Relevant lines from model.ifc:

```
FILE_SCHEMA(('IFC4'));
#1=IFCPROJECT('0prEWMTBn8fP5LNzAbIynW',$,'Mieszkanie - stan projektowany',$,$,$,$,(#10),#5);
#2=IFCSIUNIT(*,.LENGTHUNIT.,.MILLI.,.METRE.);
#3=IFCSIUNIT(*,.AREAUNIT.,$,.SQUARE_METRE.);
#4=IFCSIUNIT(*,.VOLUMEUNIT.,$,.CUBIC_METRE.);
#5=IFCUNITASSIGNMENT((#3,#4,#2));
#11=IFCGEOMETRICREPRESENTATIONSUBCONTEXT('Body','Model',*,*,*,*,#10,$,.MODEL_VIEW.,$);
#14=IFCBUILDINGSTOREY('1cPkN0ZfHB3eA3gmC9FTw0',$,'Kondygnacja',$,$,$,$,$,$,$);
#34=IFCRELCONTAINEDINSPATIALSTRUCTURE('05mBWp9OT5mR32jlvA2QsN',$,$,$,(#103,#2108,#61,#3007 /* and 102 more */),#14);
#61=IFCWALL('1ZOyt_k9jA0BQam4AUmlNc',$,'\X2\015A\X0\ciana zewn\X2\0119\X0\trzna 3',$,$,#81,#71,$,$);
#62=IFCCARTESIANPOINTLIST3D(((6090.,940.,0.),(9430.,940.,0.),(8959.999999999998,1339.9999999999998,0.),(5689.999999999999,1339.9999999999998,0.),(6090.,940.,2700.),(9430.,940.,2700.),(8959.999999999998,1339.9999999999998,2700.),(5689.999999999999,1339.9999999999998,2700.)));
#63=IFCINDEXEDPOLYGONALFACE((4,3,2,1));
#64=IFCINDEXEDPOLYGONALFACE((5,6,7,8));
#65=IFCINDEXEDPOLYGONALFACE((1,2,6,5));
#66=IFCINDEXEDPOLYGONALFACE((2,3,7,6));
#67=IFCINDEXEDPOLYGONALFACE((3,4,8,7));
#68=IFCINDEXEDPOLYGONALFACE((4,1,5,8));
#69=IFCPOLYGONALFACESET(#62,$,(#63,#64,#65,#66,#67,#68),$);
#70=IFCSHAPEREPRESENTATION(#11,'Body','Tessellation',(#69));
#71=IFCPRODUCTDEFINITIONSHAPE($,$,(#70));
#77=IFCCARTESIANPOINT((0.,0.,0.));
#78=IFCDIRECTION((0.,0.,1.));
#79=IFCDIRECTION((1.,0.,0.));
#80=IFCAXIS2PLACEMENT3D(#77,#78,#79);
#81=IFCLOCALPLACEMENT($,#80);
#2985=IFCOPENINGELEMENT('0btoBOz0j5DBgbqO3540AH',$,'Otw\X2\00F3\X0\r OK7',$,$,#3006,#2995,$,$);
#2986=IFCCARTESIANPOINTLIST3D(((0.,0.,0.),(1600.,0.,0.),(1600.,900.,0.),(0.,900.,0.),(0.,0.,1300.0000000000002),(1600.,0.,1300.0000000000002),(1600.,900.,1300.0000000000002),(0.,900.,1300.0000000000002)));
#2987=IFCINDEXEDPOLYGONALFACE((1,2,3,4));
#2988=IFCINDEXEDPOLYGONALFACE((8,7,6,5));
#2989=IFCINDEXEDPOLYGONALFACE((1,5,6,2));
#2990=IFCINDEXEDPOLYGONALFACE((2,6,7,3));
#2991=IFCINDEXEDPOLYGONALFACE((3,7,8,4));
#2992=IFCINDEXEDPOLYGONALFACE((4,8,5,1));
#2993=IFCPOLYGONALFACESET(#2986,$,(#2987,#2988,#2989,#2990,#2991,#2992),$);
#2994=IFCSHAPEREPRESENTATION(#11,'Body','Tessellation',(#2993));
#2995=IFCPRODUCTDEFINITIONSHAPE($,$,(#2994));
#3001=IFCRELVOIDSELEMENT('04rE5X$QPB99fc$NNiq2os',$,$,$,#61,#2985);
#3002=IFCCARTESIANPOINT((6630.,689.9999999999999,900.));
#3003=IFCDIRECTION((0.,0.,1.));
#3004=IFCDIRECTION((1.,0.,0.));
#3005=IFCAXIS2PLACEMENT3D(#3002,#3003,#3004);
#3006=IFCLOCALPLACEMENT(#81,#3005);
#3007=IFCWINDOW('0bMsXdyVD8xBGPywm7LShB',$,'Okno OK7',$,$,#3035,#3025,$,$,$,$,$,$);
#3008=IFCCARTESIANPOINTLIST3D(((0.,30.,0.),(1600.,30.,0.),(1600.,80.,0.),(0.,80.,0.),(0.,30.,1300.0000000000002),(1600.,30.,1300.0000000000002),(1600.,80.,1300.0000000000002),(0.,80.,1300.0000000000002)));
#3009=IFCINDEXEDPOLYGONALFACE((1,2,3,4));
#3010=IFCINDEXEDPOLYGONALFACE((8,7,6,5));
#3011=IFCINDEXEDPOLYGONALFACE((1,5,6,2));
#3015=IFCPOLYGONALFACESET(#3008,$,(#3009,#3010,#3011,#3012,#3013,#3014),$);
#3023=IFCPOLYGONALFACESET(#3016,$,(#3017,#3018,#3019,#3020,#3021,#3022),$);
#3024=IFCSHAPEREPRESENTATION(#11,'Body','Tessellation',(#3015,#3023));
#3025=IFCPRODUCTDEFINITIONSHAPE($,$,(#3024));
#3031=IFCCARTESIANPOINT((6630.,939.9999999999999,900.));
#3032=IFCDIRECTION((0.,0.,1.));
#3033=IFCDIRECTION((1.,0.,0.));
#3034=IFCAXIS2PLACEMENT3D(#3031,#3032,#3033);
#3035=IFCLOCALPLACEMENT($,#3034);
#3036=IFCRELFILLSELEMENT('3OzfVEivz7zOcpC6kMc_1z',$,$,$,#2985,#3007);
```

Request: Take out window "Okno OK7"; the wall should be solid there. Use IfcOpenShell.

```python
import ifcopenshell
import ifcopenshell.api.feature
import ifcopenshell.api.root
import ifcopenshell.geom
import ifcopenshell.util.shape

model = ifcopenshell.open("model.ifc")
settings = ifcopenshell.geom.settings()


def volume(element):
    """Net volume in cubic metres, openings subtracted."""
    shape = ifcopenshell.geom.create_shape(settings, element)
    return ifcopenshell.util.shape.get_volume(shape.geometry)


window = model.by_id(3007)
opening = window.FillsVoids[0].RelatingOpeningElement
wall = opening.VoidsElements[0].RelatingBuildingElement
before = volume(wall)

ifcopenshell.api.root.remove_product(model, product=window)
ifcopenshell.api.feature.remove_feature(model, feature=opening)

after = volume(wall)

print(f"wall volume {before:.3f} -> {after:.3f} m3")

model.write("model_updated.ifc")
```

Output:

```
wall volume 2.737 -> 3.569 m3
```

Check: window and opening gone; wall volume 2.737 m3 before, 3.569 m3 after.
